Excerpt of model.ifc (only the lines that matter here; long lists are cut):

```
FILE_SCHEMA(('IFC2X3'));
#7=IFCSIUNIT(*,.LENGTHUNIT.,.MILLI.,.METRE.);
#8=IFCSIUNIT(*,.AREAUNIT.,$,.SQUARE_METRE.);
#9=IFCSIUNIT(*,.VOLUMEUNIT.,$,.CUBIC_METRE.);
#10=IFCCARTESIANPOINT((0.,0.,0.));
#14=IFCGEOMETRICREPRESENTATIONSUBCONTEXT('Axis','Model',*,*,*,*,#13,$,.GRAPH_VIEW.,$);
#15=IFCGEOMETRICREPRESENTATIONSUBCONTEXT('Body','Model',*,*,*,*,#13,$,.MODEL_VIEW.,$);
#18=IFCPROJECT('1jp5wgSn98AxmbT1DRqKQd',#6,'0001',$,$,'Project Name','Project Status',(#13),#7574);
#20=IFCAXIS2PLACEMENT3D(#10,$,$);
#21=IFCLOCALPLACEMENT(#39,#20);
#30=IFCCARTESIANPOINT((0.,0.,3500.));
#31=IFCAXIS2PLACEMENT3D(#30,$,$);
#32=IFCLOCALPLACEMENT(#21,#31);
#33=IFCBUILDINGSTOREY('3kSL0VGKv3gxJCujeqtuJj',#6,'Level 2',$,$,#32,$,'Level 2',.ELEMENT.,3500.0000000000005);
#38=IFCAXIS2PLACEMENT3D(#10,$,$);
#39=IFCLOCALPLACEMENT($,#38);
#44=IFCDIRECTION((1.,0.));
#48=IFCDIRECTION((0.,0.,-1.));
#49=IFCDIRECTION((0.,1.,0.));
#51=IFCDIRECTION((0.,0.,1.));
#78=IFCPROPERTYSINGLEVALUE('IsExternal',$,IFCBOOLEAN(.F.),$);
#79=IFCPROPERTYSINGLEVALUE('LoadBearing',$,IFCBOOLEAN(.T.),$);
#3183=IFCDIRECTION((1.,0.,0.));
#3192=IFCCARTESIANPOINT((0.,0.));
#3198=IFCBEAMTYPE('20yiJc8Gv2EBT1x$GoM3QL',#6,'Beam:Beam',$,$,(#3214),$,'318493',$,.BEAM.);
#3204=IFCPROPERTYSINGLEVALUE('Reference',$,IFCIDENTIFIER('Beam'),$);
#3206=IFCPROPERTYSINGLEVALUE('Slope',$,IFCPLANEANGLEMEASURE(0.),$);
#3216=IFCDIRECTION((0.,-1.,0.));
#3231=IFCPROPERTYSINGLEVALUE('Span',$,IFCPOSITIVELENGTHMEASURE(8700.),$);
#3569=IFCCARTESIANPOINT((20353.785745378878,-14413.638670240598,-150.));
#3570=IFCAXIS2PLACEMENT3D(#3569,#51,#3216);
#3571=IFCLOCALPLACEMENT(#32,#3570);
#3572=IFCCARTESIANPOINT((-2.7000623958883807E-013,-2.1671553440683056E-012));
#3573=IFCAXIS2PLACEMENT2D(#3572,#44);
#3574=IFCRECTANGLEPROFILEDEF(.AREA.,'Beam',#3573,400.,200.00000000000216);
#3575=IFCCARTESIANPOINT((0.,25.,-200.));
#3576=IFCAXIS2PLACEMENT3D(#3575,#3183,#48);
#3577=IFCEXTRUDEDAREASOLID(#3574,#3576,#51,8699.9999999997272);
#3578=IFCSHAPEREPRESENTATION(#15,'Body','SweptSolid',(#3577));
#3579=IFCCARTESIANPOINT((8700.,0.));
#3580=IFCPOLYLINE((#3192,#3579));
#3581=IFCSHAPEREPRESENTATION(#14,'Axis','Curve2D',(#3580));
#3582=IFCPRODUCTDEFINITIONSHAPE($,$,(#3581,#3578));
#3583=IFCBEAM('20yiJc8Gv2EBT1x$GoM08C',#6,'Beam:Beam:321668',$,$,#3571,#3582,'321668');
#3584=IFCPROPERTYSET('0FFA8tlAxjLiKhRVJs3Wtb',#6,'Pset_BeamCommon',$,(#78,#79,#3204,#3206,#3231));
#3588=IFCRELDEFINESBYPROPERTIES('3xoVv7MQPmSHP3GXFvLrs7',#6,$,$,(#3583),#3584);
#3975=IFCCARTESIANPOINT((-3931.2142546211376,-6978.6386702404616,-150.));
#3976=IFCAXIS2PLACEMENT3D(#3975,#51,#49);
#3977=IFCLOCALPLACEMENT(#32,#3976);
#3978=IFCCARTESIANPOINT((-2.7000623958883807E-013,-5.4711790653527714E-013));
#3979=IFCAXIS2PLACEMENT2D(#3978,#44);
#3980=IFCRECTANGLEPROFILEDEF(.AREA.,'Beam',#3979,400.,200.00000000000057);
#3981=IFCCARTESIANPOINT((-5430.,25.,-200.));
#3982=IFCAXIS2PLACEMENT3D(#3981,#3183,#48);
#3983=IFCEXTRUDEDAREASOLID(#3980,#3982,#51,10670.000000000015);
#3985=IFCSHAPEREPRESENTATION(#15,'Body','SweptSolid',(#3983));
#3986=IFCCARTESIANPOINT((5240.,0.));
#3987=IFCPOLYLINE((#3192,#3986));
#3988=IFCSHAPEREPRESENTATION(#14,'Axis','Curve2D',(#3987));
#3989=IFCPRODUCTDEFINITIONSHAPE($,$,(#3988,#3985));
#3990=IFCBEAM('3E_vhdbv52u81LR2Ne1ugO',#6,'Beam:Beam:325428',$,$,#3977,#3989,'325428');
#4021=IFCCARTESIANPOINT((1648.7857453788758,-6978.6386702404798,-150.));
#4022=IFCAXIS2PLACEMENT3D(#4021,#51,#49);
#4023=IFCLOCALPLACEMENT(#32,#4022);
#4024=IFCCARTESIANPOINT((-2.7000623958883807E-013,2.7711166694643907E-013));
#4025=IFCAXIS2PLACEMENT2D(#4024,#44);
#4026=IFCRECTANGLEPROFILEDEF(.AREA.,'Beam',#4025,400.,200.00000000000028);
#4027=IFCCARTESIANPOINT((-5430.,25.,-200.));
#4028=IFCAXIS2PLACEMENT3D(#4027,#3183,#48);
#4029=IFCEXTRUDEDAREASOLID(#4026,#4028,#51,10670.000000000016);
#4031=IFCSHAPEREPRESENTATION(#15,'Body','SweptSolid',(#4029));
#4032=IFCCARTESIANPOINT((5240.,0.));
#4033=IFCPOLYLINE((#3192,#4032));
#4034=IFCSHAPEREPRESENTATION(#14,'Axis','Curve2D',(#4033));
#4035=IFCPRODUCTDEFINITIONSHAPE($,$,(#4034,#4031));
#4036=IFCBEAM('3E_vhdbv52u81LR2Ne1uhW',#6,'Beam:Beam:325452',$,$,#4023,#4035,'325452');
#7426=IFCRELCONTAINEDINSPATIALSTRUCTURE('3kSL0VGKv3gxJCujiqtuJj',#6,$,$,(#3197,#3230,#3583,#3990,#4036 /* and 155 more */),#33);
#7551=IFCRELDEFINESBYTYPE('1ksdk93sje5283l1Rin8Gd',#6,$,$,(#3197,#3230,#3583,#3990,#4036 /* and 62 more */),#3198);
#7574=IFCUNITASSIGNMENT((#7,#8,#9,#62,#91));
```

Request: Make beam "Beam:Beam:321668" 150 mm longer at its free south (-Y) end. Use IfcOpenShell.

```python
import numpy as np
import ifcopenshell
import ifcopenshell.api.pset
import ifcopenshell.util.element
import ifcopenshell.util.representation
import ifcopenshell.util.unit

model = ifcopenshell.open("model.ifc")
unit_scale = ifcopenshell.util.unit.calculate_unit_scale(model)

member = model.by_guid("20yiJc8Gv2EBT1x$GoM08C")
change = 0.15 / unit_scale

# The extrusion runs towards the end named, so only its depth changes.
body = ifcopenshell.util.representation.get_representation(member, "Model", "Body")
solid = body.Items[0]
old_length = solid.Depth
solid.Depth += change

# Move the axis end point with it.
axis = next(r for r in member.Representation.Representations if r.RepresentationIdentifier == "Axis").Items[0]
start, end = (np.array(p.Coordinates) for p in axis.Points)
end = end + (end - start) / np.linalg.norm(end - start) * change
point = model.createIfcCartesianPoint(end.tolist())
axis.Points = [axis.Points[0], point]

# Update the stored length and volume.
pset = model.by_id(ifcopenshell.util.element.get_pset(member, "Pset_BeamCommon", should_inherit=False)["id"])
ifcopenshell.api.pset.edit_pset(model, pset=pset, properties={
    "Span": model.create_entity("IfcPositiveLengthMeasure", solid.Depth),
})

print(f"length {old_length:g} -> {solid.Depth:g}")

model.write("model_updated.ifc")
```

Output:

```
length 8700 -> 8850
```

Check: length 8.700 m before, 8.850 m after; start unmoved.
